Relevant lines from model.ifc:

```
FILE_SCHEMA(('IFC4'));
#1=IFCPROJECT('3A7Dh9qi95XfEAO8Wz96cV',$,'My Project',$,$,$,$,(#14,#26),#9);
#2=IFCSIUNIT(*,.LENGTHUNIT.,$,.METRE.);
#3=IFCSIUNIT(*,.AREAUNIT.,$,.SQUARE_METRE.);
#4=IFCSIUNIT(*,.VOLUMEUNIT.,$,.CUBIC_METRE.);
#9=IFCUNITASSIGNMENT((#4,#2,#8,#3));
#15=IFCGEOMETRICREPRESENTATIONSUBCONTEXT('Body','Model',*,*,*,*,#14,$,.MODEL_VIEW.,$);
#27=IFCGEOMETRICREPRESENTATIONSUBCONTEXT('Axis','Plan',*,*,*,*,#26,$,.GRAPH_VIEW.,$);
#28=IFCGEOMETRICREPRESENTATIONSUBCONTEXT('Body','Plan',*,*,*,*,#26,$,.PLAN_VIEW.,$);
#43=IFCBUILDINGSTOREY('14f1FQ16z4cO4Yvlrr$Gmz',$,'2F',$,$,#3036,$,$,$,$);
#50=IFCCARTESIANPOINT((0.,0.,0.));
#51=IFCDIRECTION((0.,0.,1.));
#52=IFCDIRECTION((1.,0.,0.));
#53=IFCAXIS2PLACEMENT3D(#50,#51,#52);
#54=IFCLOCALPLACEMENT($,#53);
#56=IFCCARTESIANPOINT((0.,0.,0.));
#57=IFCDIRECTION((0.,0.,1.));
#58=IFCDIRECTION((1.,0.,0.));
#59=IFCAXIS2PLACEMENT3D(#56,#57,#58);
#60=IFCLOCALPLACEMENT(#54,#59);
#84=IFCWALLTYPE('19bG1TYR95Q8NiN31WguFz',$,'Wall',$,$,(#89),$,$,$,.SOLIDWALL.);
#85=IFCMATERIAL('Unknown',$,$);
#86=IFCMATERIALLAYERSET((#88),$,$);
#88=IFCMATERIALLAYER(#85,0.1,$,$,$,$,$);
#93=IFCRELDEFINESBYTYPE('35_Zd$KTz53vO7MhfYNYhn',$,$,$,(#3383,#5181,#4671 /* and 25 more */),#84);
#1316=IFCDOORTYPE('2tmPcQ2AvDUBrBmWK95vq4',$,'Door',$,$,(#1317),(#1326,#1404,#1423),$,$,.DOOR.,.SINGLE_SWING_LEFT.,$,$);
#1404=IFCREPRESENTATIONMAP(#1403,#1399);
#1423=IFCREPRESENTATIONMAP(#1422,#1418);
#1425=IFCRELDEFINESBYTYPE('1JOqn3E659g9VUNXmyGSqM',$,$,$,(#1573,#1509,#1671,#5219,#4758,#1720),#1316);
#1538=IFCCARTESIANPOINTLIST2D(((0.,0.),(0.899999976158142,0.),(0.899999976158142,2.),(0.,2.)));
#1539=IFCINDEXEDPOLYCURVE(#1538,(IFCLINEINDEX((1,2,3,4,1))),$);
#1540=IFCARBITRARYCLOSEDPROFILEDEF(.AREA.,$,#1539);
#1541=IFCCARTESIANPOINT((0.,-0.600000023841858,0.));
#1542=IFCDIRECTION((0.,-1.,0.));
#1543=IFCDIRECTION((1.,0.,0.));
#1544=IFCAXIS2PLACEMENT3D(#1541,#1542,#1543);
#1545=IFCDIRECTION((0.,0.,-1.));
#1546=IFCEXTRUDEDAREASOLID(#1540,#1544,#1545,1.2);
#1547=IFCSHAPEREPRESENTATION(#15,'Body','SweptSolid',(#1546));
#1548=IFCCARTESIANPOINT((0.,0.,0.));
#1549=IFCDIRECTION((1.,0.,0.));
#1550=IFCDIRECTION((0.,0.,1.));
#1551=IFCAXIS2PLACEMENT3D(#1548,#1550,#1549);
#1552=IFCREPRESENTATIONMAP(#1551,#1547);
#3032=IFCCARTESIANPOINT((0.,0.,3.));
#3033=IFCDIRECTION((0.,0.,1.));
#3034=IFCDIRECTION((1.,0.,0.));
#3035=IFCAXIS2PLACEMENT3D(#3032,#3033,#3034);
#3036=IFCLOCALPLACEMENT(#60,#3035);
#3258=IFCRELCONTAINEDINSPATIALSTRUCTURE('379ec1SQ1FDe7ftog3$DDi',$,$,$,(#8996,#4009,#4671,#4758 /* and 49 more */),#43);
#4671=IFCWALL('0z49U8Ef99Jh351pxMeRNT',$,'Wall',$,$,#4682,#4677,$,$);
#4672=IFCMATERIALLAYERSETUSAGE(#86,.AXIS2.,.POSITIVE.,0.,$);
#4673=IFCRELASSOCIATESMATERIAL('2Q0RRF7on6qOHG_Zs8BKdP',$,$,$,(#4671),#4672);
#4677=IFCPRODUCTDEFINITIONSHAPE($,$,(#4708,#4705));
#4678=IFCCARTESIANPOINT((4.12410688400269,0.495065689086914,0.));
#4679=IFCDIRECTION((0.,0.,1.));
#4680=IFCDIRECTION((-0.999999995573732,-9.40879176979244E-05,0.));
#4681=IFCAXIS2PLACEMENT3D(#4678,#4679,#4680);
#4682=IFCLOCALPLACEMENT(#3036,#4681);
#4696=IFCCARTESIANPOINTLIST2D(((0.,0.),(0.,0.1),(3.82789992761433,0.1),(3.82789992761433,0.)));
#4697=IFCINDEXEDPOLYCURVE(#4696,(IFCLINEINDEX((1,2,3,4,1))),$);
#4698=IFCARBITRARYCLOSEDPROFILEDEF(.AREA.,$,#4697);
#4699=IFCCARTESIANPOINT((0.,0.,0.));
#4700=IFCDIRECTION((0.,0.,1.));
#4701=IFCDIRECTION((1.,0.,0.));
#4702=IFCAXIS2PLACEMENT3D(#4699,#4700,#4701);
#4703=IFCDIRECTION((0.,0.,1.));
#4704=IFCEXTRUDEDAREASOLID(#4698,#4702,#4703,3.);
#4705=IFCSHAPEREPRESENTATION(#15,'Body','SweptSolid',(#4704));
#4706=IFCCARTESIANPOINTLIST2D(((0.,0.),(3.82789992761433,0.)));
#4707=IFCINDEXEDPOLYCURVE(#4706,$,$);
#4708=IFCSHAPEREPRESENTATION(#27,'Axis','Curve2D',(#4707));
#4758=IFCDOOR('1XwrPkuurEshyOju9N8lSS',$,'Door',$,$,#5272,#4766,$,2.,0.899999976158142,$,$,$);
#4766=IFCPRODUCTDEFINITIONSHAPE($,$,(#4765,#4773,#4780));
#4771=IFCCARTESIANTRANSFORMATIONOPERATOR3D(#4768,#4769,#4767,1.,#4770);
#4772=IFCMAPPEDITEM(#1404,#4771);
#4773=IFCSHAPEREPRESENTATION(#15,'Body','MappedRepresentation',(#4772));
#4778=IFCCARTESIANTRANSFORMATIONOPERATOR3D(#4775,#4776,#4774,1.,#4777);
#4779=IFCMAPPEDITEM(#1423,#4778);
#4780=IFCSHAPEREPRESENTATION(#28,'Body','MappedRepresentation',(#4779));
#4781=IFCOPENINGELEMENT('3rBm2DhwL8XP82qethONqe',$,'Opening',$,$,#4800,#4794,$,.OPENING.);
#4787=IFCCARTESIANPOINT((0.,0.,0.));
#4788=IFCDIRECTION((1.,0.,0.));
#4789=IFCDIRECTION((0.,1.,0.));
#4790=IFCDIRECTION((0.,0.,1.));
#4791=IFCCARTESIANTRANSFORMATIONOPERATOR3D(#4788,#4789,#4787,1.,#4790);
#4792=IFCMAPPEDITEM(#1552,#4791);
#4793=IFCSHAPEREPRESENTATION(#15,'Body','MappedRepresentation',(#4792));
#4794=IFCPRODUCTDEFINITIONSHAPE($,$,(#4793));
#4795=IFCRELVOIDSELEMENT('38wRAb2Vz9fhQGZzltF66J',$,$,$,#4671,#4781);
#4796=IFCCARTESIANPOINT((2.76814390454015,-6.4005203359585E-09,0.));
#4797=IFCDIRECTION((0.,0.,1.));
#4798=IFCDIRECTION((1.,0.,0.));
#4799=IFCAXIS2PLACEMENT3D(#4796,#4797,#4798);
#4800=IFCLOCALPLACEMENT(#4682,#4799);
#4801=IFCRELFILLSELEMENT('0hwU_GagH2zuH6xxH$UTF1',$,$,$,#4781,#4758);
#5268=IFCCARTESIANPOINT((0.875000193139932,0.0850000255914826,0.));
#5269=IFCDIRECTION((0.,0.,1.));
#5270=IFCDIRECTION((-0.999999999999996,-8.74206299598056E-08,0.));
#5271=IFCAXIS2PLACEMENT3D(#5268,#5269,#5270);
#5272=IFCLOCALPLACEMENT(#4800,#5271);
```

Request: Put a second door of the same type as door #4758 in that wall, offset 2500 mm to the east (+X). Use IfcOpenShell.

```python
import ifcopenshell
import ifcopenshell.api.feature
import ifcopenshell.api.geometry
import ifcopenshell.api.root
import ifcopenshell.geom
import ifcopenshell.util.element
import ifcopenshell.util.placement
import ifcopenshell.util.shape
import ifcopenshell.util.unit

model = ifcopenshell.open("model.ifc")
unit_scale = ifcopenshell.util.unit.calculate_unit_scale(model)
settings = ifcopenshell.geom.settings()


def volume(element):
    """Net volume in cubic metres, openings subtracted."""
    shape = ifcopenshell.geom.create_shape(settings, element)
    return ifcopenshell.util.shape.get_volume(shape.geometry)


door = model.by_guid("1XwrPkuurEshyOju9N8lSS")
opening = door.FillsVoids[0].RelatingOpeningElement
wall = opening.VoidsElements[0].RelatingBuildingElement
before = volume(wall)
shift = ifcopenshell.util.placement.get_local_placement(wall.ObjectPlacement)[:3, 0] * -2.5 / unit_scale

# copy_class copies the void relationship, type, container and properties, but no geometry.
new_opening = ifcopenshell.api.root.copy_class(model, product=opening)
new_opening.Representation = ifcopenshell.util.element.copy_deep(
    model, opening.Representation, exclude=["IfcGeometricRepresentationContext", "IfcRepresentationMap"]
)
new_door = ifcopenshell.api.root.copy_class(model, product=door)
new_door.Representation = ifcopenshell.util.element.copy_deep(
    model, door.Representation, exclude=["IfcGeometricRepresentationContext", "IfcRepresentationMap"]
)
ifcopenshell.api.feature.add_filling(model, opening=new_opening, element=new_door)

for old, new in ((opening, new_opening), (door, new_door)):
    matrix = ifcopenshell.util.placement.get_local_placement(old.ObjectPlacement)
    matrix[:3, 3] += shift
    ifcopenshell.api.geometry.edit_object_placement(model, product=new, matrix=matrix, is_si=False)

after = volume(wall)

print(f"wall volume {before:.3f} -> {after:.3f} m3")

model.write("model-out.ifc")
```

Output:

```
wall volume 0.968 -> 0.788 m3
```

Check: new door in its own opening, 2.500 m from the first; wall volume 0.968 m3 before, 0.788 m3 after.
